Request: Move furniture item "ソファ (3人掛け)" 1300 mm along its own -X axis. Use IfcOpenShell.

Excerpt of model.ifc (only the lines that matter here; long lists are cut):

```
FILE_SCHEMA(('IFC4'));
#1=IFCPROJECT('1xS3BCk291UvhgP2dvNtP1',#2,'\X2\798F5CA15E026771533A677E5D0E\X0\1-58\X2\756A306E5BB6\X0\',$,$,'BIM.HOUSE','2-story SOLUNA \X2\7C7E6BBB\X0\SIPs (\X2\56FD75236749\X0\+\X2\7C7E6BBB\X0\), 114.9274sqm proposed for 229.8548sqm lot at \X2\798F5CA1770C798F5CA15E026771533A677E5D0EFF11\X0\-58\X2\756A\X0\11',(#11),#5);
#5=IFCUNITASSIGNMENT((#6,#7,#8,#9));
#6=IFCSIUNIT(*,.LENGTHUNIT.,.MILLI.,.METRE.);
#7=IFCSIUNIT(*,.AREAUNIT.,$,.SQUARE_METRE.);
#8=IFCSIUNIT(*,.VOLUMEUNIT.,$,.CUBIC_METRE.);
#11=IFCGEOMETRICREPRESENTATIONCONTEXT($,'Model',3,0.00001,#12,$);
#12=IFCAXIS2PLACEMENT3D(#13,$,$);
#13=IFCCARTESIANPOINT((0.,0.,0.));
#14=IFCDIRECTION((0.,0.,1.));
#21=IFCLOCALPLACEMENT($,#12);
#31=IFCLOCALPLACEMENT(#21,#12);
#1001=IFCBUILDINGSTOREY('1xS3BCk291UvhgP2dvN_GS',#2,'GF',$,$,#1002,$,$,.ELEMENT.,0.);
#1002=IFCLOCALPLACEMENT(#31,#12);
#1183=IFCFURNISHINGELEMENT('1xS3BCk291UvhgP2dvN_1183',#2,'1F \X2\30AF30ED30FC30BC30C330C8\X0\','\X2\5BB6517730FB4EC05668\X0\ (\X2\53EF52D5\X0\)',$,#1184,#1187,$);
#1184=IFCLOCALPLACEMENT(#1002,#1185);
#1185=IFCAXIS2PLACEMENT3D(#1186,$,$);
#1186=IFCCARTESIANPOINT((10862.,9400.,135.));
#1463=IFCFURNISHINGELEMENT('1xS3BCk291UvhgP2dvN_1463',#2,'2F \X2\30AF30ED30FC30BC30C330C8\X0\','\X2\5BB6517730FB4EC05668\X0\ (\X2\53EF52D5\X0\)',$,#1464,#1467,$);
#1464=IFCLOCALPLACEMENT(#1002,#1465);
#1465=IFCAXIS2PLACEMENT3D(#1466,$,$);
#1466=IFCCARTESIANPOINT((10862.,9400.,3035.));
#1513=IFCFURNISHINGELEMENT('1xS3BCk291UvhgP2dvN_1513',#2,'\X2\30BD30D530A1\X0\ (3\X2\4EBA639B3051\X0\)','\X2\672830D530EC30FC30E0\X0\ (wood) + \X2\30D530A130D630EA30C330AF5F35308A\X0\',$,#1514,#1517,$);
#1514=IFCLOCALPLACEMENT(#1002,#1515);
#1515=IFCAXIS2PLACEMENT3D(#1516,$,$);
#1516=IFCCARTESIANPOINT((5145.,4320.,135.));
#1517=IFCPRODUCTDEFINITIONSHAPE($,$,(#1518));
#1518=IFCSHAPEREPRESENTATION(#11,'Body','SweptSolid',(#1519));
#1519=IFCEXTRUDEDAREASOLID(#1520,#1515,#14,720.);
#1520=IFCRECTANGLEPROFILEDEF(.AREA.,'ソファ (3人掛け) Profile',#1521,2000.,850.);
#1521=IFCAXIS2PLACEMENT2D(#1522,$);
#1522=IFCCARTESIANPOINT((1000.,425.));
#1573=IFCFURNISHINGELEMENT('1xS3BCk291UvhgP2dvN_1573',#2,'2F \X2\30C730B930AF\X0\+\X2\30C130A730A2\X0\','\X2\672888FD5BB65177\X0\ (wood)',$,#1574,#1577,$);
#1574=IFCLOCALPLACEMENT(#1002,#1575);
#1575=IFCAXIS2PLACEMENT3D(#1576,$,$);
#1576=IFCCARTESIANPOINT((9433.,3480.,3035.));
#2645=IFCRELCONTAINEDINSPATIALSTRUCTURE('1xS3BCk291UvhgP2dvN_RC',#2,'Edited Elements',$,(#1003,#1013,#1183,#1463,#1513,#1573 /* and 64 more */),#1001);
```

```python
import ifcopenshell
import ifcopenshell.api.geometry
import ifcopenshell.util.placement
import ifcopenshell.util.unit

model = ifcopenshell.open("model.ifc")
unit_scale = ifcopenshell.util.unit.calculate_unit_scale(model)

item = model.by_id(1513)
matrix = ifcopenshell.util.placement.get_local_placement(item.ObjectPlacement)
matrix[:3, 3] -= matrix[:3, 0] * 1.3 / unit_scale
ifcopenshell.api.geometry.edit_object_placement(model, product=item, matrix=matrix, is_si=False)

print(ifcopenshell.util.placement.get_local_placement(item.ObjectPlacement).round(3) + 0.0)

model.write("model-out.ifc")
```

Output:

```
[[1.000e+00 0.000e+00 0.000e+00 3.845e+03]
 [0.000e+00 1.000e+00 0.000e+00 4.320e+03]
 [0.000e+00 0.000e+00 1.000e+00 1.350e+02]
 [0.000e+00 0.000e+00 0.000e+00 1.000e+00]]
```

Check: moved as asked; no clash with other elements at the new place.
